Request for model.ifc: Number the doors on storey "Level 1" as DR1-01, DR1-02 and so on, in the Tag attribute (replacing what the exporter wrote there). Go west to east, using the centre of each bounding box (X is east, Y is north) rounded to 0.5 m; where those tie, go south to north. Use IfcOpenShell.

First a look at what the model holds.

```python
import ifcopenshell
import ifcopenshell.util.element
import ifcopenshell.util.placement

model = ifcopenshell.open("model.ifc")
print(model.schema)
storey = next(s for s in model.by_type("IfcBuildingStorey") if s.Name == "Level 1")
doors = [e for e in ifcopenshell.util.element.get_decomposition(storey) if e.is_a("IfcDoor")]
for e in sorted(doors, key=lambda e: e.id()):
    origin = ifcopenshell.util.placement.get_local_placement(e.ObjectPlacement)[:3, 3]
    print(e.id(), e.Tag, e.Name, origin.round(2) + 0.0, sep=" | ")
```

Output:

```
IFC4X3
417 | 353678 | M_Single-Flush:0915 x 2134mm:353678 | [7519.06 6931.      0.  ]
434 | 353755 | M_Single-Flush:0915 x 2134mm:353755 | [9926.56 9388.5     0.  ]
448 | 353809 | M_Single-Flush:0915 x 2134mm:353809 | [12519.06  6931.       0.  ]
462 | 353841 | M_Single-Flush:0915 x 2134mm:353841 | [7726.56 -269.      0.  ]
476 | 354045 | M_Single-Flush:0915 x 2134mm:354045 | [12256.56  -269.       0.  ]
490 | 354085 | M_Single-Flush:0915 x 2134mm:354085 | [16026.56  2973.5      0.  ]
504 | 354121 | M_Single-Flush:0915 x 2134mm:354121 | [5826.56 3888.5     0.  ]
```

```python
import ifcopenshell
import ifcopenshell.geom
import ifcopenshell.util.element
import ifcopenshell.util.shape

model = ifcopenshell.open("model.ifc")
settings = ifcopenshell.geom.settings()
settings.set("use-world-coords", True)


def centre(element):
    shape = ifcopenshell.geom.create_shape(settings, element)
    return ifcopenshell.util.shape.get_bbox_centroid(shape.geometry)


storey = next(s for s in model.by_type("IfcBuildingStorey") if s.Name == "Level 1")
doors = [e for e in ifcopenshell.util.element.get_decomposition(storey) if e.is_a("IfcDoor")]

# Insertion points can sit at a corner or the storey origin, so sort by the geometry (in metres).
centres = {e: centre(e) for e in doors}
doors.sort(key=lambda e: (round(centres[e][0] / 0.5), centres[e][1]))

for i, e in enumerate(doors, start=1):
    number = f"DR1-{i:02d}"
    e.Tag = number
    print(e.id(), number)

model.write("model_rev.ifc")
```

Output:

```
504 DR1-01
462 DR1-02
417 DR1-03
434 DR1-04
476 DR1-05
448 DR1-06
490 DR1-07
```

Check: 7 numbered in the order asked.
